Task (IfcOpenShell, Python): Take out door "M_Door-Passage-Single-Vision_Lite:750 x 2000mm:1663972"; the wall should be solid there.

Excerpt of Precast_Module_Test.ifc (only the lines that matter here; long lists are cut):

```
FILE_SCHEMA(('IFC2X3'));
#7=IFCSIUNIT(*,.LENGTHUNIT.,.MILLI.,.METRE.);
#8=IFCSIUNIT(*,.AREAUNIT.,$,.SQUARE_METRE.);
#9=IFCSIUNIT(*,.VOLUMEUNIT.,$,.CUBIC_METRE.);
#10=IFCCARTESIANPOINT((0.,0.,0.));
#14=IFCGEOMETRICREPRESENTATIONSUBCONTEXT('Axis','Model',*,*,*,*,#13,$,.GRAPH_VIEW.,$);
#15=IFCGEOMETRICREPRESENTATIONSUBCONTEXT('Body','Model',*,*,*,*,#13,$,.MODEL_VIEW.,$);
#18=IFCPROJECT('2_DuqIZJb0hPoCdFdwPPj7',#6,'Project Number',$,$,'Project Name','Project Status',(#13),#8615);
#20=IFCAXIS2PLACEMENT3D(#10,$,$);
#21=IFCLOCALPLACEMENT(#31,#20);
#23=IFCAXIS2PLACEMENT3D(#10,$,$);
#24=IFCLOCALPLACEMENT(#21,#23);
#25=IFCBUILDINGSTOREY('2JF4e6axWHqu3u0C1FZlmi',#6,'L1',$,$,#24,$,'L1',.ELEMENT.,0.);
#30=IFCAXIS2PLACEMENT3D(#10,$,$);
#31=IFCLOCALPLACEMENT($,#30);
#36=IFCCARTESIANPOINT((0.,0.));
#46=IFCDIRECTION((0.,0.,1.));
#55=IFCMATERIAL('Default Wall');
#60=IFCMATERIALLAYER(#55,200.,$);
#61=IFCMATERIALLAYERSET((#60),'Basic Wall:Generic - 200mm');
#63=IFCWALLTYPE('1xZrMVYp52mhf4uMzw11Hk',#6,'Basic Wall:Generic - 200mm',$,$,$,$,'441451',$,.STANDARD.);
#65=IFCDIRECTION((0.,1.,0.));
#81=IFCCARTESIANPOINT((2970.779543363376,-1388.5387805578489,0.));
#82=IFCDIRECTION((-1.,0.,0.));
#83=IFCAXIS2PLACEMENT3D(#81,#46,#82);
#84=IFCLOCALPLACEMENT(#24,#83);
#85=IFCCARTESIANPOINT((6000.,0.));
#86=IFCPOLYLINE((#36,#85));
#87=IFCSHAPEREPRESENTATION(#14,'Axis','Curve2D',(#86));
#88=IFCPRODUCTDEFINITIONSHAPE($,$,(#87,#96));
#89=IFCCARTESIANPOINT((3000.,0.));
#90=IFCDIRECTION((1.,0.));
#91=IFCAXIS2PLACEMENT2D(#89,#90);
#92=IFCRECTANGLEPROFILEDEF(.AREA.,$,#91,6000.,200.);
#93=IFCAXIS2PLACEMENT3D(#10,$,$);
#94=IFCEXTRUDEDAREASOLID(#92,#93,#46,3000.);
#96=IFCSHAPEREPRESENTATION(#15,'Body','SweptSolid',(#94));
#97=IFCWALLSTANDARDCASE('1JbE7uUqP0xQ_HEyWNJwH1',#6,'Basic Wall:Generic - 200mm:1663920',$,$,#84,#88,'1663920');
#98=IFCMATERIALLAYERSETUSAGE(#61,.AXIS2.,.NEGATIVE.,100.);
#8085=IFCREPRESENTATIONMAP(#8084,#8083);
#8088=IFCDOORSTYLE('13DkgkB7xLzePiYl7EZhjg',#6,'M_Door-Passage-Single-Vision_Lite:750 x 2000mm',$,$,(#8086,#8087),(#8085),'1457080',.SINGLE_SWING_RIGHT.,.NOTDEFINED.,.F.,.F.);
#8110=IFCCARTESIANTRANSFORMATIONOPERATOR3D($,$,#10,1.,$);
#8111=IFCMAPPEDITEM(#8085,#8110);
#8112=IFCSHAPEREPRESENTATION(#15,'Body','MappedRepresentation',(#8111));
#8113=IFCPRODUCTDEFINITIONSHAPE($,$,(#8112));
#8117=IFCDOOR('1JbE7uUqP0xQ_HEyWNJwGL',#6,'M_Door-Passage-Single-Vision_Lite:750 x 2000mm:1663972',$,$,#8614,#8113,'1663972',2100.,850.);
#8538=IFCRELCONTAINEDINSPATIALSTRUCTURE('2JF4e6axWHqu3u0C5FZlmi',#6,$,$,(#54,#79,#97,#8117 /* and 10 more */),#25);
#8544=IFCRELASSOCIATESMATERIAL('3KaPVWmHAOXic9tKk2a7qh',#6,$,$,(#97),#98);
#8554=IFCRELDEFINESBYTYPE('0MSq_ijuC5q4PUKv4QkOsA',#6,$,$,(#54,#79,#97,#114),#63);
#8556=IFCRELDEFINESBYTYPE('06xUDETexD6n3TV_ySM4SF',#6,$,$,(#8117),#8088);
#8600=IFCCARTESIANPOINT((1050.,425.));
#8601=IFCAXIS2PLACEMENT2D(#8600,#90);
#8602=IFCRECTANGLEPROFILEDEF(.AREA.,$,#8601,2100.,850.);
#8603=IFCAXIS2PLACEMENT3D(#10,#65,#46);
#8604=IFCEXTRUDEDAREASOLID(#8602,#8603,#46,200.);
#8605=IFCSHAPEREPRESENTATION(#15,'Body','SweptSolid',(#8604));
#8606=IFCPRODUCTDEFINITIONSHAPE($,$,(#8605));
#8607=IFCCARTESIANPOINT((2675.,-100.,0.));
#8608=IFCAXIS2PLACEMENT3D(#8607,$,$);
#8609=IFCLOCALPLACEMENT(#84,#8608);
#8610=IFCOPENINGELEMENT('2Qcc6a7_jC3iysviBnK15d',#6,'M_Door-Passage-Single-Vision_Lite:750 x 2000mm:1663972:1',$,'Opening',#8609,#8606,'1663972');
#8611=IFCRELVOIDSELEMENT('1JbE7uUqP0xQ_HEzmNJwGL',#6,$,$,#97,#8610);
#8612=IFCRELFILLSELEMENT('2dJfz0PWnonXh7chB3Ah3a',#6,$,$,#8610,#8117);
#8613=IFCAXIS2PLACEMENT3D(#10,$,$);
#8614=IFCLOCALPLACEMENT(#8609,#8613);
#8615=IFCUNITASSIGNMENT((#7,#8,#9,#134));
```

```python
import ifcopenshell
import ifcopenshell.api.feature
import ifcopenshell.api.root
import ifcopenshell.geom
import ifcopenshell.util.shape

model = ifcopenshell.open("Precast_Module_Test.ifc")
settings = ifcopenshell.geom.settings()


def volume(element):
    """Net volume in cubic metres, openings subtracted."""
    shape = ifcopenshell.geom.create_shape(settings, element)
    return ifcopenshell.util.shape.get_volume(shape.geometry)


door = model.by_guid("1JbE7uUqP0xQ_HEyWNJwGL")
opening = door.FillsVoids[0].RelatingOpeningElement
wall = opening.VoidsElements[0].RelatingBuildingElement
before = volume(wall)

ifcopenshell.api.root.remove_product(model, product=door)
ifcopenshell.api.feature.remove_feature(model, feature=opening)

after = volume(wall)

print(f"wall volume {before:.3f} -> {after:.3f} m3")

model.write("Precast_Module_Test_rev.ifc")
```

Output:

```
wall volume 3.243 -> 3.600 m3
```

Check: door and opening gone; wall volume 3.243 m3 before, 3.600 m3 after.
